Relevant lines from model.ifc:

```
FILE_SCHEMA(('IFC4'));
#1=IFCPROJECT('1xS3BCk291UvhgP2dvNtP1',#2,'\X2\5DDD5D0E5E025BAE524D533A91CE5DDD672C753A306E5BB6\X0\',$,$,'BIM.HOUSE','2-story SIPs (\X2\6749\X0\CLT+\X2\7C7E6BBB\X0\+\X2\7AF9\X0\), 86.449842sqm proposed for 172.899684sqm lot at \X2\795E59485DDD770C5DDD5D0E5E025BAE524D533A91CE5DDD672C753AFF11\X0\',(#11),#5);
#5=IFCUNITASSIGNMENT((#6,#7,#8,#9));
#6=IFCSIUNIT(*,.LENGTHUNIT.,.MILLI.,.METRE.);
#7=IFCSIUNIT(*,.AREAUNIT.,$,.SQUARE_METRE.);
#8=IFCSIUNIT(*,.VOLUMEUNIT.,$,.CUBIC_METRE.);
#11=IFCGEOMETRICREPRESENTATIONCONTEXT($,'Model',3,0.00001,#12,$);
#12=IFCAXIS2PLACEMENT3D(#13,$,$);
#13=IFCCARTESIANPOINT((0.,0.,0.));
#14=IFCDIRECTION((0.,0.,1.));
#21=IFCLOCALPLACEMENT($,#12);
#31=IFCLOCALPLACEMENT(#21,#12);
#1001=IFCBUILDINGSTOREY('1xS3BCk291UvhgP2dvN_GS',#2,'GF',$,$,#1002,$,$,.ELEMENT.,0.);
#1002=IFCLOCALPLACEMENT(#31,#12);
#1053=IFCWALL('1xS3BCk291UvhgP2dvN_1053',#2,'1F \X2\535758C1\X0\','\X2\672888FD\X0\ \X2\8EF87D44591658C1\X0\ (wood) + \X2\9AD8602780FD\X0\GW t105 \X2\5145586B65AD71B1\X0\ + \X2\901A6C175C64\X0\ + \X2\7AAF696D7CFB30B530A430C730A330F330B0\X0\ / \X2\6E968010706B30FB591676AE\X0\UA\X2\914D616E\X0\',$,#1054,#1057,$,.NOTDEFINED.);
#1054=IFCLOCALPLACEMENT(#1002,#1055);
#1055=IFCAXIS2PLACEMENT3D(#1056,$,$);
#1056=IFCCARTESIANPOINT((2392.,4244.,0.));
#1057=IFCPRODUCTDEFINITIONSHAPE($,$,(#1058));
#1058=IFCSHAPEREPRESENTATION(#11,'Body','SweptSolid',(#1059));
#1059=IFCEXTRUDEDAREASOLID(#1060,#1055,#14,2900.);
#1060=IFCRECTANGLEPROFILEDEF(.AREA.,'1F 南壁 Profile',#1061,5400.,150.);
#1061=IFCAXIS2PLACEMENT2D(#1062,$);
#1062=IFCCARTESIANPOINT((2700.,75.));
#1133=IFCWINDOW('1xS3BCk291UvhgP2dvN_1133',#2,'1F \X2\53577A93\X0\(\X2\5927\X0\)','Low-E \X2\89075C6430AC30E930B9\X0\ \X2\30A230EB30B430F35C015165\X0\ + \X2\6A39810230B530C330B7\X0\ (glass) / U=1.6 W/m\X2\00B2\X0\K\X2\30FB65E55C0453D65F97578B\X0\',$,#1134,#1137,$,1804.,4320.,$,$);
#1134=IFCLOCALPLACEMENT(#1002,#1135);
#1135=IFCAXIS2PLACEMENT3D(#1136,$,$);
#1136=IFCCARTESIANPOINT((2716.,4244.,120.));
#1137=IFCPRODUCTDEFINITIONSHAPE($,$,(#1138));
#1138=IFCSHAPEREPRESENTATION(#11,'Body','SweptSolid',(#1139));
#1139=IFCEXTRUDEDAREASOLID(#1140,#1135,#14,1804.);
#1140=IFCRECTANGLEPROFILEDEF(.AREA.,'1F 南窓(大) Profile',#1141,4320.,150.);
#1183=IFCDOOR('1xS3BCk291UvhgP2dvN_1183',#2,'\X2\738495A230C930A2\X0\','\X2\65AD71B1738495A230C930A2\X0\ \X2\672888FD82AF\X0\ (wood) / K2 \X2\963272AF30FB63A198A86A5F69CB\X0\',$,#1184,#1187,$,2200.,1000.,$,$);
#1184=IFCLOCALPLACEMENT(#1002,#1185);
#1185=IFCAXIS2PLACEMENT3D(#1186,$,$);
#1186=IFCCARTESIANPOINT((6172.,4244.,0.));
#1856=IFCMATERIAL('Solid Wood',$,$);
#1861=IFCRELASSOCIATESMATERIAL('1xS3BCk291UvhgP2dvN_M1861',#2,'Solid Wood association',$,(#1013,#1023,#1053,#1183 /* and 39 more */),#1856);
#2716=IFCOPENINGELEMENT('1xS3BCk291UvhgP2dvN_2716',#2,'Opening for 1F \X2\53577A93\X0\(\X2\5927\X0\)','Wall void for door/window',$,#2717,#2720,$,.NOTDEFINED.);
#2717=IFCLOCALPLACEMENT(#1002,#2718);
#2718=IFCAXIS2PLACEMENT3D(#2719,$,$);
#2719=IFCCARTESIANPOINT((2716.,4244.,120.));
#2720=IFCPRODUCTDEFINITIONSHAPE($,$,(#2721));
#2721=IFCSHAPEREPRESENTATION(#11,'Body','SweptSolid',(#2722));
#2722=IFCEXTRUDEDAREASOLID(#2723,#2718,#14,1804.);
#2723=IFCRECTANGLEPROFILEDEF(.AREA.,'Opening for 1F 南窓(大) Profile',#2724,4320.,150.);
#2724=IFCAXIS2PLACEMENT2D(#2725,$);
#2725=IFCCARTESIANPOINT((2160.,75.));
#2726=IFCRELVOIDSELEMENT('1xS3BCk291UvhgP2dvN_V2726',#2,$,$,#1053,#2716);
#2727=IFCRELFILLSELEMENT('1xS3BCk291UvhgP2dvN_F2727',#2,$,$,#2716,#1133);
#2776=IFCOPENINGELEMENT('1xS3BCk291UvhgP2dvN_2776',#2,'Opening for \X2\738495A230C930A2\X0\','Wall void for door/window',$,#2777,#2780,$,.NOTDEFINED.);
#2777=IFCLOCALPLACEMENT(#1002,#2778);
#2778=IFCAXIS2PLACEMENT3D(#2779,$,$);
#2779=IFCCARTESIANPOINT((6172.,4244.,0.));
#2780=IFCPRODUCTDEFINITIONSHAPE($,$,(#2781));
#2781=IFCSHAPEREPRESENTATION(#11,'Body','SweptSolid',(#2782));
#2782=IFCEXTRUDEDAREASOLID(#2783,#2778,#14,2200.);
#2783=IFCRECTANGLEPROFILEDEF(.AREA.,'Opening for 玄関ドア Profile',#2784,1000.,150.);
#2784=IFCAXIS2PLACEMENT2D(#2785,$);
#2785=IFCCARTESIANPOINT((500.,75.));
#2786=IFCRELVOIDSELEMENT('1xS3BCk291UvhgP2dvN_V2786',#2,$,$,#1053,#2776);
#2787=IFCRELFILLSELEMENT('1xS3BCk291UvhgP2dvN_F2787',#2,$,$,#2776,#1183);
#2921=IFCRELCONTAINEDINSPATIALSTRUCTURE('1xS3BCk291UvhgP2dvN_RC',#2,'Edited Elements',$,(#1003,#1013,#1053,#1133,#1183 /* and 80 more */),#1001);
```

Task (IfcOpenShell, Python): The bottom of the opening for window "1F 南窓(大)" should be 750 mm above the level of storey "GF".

```python
import numpy as np
import ifcopenshell
import ifcopenshell.api.geometry
import ifcopenshell.geom
import ifcopenshell.util.element
import ifcopenshell.util.placement
import ifcopenshell.util.shape
import ifcopenshell.util.unit

model = ifcopenshell.open("model.ifc")
unit_scale = ifcopenshell.util.unit.calculate_unit_scale(model)

window = model.by_guid("1xS3BCk291UvhgP2dvN_1133")
opening = window.FillsVoids[0].RelatingOpeningElement
storey = ifcopenshell.util.element.get_container(window, ifc_class="IfcBuildingStorey")
level = ifcopenshell.util.placement.get_local_placement(storey.ObjectPlacement)[2, 3]

# The opening's origin need not be at the sill, so measure its lowest point.
shape = ifcopenshell.geom.create_shape(ifcopenshell.geom.settings(), opening)
bottom = ifcopenshell.util.shape.get_shape_bottom_elevation(shape, shape.geometry) / unit_scale
dz = level + 0.75 / unit_scale - bottom

shift = np.array([0.0, 0.0, dz])
# The window is not placed relative to its opening, so move both.
for product in (opening, window):
    matrix = ifcopenshell.util.placement.get_local_placement(product.ObjectPlacement)
    matrix[:3, 3] += shift
    ifcopenshell.api.geometry.edit_object_placement(model, product=product, matrix=matrix, is_si=False)

print(f"moved by {dz * unit_scale:+.3f} m")

model.write("model_v2.ifc")
```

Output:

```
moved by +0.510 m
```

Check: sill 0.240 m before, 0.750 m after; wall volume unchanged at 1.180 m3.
